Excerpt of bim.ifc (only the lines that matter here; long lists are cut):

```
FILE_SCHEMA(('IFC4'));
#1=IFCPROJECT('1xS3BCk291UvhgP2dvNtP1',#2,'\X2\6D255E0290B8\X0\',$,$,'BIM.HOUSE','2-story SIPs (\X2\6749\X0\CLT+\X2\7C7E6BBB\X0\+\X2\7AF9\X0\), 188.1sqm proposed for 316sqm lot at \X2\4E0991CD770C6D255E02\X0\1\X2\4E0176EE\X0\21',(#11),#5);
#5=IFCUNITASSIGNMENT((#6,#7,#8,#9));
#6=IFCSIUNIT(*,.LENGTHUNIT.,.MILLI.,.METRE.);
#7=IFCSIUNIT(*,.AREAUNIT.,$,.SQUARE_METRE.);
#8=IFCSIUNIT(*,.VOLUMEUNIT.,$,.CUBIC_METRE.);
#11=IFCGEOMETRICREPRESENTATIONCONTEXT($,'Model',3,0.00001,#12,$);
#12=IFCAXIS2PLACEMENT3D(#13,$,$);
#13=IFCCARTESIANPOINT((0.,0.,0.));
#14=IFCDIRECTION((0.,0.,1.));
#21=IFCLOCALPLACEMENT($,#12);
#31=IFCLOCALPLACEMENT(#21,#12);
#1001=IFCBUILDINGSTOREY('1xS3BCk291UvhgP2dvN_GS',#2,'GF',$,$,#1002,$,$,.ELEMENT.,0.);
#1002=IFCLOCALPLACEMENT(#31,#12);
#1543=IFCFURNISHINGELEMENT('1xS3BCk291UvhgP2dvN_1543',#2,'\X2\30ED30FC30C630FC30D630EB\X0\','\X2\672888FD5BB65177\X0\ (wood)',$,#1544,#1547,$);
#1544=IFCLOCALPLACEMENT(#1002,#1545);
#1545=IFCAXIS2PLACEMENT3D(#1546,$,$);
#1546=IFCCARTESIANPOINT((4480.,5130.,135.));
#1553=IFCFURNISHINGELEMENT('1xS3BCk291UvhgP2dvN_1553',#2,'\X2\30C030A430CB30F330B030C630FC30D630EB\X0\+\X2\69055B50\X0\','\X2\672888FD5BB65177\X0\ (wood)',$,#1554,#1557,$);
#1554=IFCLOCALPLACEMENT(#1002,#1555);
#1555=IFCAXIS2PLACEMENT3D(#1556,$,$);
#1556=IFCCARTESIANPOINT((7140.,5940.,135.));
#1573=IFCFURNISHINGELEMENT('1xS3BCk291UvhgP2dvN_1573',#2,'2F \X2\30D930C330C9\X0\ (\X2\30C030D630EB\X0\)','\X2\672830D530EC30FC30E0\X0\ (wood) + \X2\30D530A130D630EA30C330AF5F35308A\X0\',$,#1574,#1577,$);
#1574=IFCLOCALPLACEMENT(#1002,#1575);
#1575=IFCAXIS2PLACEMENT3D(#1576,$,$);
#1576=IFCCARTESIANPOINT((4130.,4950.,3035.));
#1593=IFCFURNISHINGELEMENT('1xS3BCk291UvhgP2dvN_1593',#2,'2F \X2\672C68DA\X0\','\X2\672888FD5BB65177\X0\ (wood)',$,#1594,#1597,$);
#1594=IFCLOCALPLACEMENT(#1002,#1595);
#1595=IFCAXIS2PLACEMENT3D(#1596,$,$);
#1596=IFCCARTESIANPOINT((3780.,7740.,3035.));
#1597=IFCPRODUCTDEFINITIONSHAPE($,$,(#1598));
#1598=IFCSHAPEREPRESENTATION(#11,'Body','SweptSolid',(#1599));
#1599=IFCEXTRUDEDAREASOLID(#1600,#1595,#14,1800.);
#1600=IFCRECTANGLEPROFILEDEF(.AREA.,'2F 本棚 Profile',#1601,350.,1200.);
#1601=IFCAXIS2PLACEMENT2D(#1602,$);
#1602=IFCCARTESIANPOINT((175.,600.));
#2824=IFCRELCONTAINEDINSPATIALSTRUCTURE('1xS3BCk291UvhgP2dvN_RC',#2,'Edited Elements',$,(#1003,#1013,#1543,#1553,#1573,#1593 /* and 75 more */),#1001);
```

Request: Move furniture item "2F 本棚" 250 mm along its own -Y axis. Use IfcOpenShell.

```python
import ifcopenshell
import ifcopenshell.api.geometry
import ifcopenshell.util.placement

model = ifcopenshell.open("bim.ifc")

item = model.by_id(1593)
matrix = ifcopenshell.util.placement.get_local_placement(item.ObjectPlacement)
matrix[:3, 3] -= matrix[:3, 1] * 250.0
ifcopenshell.api.geometry.edit_object_placement(model, product=item, matrix=matrix, is_si=False)

print(ifcopenshell.util.placement.get_local_placement(item.ObjectPlacement).round(3) + 0.0)

model.write("bim_updated.ifc")
```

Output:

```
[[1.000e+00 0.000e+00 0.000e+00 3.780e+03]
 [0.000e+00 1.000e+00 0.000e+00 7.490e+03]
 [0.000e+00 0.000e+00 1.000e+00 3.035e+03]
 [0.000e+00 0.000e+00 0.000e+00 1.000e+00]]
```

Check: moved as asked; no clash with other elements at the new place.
